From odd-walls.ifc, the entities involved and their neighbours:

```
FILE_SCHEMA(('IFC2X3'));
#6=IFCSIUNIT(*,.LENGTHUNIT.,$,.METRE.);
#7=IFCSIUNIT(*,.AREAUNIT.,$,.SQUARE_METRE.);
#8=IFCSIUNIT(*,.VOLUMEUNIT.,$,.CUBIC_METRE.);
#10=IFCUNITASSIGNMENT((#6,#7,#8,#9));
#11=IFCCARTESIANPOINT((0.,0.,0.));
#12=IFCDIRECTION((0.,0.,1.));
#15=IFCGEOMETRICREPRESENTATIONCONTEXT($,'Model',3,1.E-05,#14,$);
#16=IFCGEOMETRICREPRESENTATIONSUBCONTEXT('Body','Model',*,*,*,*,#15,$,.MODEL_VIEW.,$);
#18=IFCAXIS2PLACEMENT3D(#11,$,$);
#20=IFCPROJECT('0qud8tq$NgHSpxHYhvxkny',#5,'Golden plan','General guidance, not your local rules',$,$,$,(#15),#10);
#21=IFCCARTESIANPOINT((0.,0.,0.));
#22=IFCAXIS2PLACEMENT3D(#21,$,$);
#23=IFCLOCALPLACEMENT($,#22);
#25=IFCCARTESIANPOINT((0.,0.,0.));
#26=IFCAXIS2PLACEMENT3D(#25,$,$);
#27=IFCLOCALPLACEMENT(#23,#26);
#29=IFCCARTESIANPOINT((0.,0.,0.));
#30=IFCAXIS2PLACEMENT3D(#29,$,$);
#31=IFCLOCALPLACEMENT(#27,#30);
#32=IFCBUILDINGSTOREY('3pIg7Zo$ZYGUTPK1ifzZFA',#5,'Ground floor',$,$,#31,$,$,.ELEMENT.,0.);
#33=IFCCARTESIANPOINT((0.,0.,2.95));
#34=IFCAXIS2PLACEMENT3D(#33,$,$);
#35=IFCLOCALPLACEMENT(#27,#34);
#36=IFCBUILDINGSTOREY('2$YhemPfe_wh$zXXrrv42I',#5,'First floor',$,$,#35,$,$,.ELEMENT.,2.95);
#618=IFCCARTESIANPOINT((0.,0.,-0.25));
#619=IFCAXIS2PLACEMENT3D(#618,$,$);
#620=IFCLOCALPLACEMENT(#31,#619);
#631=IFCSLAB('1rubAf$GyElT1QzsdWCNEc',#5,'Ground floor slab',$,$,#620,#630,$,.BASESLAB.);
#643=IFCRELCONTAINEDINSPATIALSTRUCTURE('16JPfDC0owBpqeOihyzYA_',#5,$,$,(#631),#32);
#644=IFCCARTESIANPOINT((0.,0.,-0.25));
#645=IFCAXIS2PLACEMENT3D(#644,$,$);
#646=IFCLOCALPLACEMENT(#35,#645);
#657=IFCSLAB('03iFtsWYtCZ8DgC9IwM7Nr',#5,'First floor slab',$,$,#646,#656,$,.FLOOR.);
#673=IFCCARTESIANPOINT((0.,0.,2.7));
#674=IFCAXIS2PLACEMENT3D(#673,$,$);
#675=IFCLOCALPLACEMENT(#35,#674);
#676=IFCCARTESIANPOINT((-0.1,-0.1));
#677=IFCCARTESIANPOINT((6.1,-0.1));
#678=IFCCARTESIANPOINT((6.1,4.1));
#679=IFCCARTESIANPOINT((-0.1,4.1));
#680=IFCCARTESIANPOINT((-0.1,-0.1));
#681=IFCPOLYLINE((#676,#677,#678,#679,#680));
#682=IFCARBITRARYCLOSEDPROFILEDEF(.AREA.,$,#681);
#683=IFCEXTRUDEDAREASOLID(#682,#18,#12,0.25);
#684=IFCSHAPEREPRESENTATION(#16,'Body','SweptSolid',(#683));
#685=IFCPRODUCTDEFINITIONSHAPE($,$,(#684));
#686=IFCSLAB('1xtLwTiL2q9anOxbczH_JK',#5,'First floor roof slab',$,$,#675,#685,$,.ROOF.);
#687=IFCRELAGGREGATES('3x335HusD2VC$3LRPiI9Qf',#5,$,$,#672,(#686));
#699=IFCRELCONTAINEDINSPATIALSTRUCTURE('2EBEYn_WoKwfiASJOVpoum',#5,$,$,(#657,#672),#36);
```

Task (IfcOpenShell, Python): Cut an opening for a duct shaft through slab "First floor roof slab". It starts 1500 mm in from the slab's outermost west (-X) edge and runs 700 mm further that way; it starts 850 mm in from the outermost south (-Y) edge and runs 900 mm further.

```python
import numpy as np
import ifcopenshell
import ifcopenshell.api.feature
import ifcopenshell.api.geometry
import ifcopenshell.api.root
import ifcopenshell.geom
import ifcopenshell.util.placement
import ifcopenshell.util.representation
import ifcopenshell.util.shape
import ifcopenshell.util.unit

model = ifcopenshell.open("odd-walls.ifc")
unit_scale = ifcopenshell.util.unit.calculate_unit_scale(model)
settings = ifcopenshell.geom.settings()


def volume(element):
    """Net volume in cubic metres, openings subtracted."""
    shape = ifcopenshell.geom.create_shape(settings, element)
    return ifcopenshell.util.shape.get_volume(shape.geometry)


slab = model.by_guid("1xtLwTiL2q9anOxbczH_JK")
before = volume(slab)

# Extent in the slab's own axes, in metres. The edges named are its -X and -Y sides.
slab_shape = ifcopenshell.geom.create_shape(settings, slab)
vertices = ifcopenshell.util.shape.get_vertices(slab_shape.geometry)
x_min, y_min, bottom = vertices.min(axis=0)
top = vertices[:, 2].max()

opening = ifcopenshell.api.root.create_entity(model, ifc_class="IfcOpeningElement", name="Duct shaft opening")
context = ifcopenshell.util.representation.get_context(model, "Model", "Body", "MODEL_VIEW")
width, depth = 0.7, 0.9
outline = [(0.0, 0.0), (width, 0.0), (width, depth), (0.0, depth), (0.0, 0.0)]
# Overshoot both faces by 50 mm so the cut is clean.
shape = ifcopenshell.api.geometry.add_slab_representation(
    model, context=context, depth=top - bottom + 0.1, polyline=outline
)
ifcopenshell.api.geometry.assign_representation(model, product=opening, representation=shape)

matrix = ifcopenshell.util.placement.get_local_placement(slab.ObjectPlacement)
matrix[:, 3] = matrix @ np.append(np.array([x_min + 1.5, y_min + 0.85, bottom - 0.05]) / unit_scale, 1.0)
ifcopenshell.api.geometry.edit_object_placement(model, product=opening, matrix=matrix, is_si=False)
ifcopenshell.api.feature.add_feature(model, feature=opening, element=slab)

after = volume(slab)

print(f"slab volume {before:.3f} -> {after:.3f} m3")

model.write("odd-walls_v2.ifc")
```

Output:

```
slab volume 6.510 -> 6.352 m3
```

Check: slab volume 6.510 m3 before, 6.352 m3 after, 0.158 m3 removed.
